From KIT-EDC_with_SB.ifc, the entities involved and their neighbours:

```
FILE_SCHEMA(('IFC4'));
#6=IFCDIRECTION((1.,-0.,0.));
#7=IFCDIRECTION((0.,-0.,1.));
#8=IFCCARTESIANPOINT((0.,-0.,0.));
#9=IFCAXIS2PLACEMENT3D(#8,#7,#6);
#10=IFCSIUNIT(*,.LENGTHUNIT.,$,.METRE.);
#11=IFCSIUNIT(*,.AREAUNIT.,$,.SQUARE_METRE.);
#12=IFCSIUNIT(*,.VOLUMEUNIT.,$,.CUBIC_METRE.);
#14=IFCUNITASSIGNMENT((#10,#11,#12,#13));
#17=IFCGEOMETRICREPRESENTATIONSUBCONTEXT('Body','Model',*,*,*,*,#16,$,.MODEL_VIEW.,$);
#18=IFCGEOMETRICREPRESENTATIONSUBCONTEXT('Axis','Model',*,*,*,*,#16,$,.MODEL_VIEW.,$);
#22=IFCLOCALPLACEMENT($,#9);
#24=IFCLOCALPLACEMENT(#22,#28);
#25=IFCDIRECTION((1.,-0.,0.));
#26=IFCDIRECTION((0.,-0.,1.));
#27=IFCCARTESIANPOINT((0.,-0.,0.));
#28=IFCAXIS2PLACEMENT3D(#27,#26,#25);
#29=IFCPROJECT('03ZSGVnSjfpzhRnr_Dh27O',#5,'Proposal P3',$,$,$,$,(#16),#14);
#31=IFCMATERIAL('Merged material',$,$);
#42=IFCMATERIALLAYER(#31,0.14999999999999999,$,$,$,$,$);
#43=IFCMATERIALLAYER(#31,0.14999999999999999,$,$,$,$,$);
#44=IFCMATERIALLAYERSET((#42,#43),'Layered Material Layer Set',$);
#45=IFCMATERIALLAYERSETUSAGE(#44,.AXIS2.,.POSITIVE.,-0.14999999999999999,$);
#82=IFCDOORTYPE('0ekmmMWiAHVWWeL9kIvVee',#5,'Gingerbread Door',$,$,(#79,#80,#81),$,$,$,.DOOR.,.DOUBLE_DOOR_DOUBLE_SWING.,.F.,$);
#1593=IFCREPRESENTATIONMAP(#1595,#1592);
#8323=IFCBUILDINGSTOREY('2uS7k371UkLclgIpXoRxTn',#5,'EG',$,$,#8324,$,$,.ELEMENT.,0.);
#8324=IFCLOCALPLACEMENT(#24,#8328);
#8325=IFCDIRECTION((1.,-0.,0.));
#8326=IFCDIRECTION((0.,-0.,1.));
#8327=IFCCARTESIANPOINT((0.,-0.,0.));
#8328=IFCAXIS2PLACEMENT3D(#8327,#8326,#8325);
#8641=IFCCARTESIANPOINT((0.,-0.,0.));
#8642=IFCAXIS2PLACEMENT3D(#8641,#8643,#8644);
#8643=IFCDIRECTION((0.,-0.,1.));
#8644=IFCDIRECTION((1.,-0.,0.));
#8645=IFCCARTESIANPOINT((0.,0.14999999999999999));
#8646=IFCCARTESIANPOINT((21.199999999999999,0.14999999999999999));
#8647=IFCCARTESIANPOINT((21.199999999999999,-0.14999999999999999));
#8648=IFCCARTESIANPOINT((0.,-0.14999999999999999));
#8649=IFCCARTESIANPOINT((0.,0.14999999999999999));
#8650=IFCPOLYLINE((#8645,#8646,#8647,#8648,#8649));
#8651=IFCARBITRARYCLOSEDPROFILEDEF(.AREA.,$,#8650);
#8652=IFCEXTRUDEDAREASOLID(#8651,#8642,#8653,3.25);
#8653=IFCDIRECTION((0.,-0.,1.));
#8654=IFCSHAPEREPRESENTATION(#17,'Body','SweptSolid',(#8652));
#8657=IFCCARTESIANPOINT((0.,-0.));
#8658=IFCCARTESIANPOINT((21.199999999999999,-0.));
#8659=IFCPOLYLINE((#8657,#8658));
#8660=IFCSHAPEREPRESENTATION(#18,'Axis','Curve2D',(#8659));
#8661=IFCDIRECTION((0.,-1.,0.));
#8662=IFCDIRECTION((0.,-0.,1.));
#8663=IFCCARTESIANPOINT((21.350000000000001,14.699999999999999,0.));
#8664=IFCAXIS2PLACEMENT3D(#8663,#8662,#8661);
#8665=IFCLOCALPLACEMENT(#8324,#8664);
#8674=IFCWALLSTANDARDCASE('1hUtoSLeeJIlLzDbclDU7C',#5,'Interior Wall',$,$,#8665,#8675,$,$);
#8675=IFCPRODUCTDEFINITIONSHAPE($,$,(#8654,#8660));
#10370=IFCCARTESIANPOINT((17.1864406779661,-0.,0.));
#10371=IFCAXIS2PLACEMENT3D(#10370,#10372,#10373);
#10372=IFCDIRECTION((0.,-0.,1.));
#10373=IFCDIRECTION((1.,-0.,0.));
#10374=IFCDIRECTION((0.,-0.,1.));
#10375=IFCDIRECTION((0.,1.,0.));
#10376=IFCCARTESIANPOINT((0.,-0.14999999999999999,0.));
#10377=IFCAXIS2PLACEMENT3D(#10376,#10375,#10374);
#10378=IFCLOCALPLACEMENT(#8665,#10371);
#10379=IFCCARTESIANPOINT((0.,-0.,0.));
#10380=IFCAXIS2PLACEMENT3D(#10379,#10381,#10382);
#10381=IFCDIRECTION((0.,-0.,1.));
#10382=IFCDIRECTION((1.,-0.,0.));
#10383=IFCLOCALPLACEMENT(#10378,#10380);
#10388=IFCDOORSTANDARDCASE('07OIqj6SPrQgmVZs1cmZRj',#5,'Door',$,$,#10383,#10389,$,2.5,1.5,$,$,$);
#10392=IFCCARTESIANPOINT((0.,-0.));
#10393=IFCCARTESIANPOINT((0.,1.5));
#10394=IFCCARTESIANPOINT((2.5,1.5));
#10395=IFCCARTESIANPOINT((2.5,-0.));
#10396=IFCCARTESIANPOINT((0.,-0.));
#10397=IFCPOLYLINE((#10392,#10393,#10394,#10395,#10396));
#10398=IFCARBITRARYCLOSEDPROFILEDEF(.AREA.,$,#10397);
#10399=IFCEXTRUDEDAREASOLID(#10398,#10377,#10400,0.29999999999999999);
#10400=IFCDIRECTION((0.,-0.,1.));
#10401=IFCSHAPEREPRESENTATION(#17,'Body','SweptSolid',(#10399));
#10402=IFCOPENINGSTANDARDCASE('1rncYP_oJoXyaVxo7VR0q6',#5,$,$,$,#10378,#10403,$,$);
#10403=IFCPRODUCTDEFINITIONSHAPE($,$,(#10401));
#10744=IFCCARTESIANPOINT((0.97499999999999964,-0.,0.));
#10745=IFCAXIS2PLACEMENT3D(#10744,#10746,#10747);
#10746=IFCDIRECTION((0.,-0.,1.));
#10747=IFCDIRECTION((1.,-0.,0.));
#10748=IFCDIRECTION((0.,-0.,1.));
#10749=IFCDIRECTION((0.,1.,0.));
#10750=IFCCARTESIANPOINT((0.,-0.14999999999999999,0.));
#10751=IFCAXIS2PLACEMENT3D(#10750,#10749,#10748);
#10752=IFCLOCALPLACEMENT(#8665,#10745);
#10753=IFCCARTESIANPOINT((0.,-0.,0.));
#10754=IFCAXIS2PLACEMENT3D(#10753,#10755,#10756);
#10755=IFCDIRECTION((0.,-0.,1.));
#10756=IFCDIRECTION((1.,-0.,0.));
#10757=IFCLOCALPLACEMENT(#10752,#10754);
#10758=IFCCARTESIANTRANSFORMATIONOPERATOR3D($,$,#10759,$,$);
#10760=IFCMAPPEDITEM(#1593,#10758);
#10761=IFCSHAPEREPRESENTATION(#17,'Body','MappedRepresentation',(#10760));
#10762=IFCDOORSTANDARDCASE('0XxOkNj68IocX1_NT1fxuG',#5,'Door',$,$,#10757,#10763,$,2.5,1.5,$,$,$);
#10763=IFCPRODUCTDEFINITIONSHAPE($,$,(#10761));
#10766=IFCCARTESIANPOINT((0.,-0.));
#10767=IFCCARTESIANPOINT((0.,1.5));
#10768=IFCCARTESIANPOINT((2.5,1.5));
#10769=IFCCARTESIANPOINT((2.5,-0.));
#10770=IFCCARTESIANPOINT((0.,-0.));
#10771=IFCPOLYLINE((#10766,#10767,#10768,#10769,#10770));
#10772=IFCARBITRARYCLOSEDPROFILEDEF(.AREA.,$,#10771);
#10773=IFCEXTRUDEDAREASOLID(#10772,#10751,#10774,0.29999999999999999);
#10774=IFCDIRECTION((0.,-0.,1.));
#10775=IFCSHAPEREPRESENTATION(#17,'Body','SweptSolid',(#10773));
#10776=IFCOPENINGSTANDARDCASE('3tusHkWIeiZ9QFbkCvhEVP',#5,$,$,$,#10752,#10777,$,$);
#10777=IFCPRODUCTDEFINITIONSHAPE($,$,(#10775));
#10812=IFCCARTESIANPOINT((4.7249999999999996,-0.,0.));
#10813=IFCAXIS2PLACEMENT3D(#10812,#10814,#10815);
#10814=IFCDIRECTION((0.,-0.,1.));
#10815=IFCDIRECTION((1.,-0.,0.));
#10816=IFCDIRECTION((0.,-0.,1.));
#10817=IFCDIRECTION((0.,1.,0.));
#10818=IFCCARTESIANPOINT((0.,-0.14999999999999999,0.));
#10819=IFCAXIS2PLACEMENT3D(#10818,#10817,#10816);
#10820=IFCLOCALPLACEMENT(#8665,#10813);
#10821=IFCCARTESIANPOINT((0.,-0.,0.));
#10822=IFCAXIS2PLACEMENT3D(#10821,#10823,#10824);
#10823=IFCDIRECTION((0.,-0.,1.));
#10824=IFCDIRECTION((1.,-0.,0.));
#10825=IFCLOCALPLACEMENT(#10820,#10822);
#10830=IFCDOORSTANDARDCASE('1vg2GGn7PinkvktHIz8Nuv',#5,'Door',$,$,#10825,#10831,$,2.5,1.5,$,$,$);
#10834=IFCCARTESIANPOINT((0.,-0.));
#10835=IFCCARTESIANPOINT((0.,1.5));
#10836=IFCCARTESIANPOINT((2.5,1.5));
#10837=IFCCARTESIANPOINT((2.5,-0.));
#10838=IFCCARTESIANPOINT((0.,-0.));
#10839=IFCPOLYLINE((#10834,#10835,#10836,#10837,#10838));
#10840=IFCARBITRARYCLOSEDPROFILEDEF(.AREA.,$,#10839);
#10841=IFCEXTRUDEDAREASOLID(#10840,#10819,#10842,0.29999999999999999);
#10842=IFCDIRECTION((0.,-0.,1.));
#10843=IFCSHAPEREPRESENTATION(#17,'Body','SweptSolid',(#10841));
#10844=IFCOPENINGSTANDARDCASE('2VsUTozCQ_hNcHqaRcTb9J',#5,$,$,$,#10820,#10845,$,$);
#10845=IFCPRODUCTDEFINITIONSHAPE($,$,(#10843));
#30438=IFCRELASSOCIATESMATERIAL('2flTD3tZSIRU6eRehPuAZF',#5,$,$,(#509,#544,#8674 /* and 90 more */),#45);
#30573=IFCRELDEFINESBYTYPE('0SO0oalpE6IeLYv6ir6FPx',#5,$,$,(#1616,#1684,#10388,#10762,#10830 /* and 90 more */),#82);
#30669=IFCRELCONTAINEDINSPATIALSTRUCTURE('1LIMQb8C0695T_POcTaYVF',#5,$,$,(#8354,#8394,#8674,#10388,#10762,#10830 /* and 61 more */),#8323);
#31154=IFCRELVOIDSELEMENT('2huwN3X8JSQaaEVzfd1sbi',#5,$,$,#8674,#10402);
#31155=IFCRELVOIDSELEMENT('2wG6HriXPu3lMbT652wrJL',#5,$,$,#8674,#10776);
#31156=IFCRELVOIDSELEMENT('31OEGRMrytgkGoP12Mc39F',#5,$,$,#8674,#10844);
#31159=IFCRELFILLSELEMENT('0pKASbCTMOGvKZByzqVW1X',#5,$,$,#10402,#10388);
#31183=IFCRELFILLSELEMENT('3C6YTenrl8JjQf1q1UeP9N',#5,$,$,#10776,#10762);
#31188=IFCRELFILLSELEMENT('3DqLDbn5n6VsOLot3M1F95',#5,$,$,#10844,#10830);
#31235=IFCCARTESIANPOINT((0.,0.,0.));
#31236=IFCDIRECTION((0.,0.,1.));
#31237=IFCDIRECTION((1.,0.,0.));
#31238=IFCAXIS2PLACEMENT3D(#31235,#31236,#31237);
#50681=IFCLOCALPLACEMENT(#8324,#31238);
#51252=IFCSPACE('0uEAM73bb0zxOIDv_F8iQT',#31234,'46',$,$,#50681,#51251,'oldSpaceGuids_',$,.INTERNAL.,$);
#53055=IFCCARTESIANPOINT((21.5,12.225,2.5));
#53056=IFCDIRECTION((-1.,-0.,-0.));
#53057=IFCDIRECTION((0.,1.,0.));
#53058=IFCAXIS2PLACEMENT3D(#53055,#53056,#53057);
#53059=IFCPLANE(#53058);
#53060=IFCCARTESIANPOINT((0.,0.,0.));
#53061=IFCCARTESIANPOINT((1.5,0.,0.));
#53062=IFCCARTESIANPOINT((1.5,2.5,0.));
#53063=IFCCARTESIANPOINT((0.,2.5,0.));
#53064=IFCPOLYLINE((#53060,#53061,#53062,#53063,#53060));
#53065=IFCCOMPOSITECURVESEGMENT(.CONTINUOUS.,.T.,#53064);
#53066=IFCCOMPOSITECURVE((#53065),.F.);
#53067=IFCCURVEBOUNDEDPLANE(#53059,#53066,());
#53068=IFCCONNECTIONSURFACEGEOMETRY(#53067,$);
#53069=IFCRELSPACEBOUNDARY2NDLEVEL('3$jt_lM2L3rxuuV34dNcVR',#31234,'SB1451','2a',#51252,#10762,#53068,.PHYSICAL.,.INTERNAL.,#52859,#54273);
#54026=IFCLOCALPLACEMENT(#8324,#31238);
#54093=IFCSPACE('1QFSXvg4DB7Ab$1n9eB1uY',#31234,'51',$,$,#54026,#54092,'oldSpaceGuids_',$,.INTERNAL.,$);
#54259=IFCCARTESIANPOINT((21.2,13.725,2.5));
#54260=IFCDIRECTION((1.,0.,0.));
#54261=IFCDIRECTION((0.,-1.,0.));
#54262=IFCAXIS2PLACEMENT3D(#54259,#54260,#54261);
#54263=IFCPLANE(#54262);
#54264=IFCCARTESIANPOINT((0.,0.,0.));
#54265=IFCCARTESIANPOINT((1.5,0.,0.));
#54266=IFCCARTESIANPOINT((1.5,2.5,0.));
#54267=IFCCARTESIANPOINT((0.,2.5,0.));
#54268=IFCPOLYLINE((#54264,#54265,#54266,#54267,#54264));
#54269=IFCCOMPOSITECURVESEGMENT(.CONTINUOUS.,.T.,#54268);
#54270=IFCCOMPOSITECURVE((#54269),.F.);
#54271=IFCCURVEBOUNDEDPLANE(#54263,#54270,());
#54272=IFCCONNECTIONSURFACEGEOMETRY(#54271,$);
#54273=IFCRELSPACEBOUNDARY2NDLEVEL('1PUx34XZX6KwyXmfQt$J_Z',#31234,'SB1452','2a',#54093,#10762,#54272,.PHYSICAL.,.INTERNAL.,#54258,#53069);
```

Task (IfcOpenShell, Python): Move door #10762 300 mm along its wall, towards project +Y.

```python
import numpy as np
import ifcopenshell
import ifcopenshell.api.geometry
import ifcopenshell.util.placement

model = ifcopenshell.open("KIT-EDC_with_SB.ifc")

door = model.by_guid("0XxOkNj68IocX1_NT1fxuG")
opening = door.FillsVoids[0].RelatingOpeningElement
wall = opening.VoidsElements[0].RelatingBuildingElement

wall_matrix = ifcopenshell.util.placement.get_local_placement(wall.ObjectPlacement)
shift = wall_matrix[:3, 0] * -0.3
before = ifcopenshell.util.placement.get_local_placement(door.ObjectPlacement)[:3, 3].copy()

# The door is placed relative to its opening, so it follows when the opening moves.
matrix = ifcopenshell.util.placement.get_local_placement(opening.ObjectPlacement)
matrix[:3, 3] += shift
ifcopenshell.api.geometry.edit_object_placement(
    model, product=opening, matrix=matrix, is_si=False, should_transform_children=True
)

# Space boundary surfaces are stored in each space's coordinates; move them too.
for rel in door.ProvidesBoundaries:
    if not rel.ConnectionGeometry:
        continue
    surface = rel.ConnectionGeometry.SurfaceOnRelatingElement.BasisSurface
    space_matrix = ifcopenshell.util.placement.get_local_placement(rel.RelatingSpace.ObjectPlacement)
    point = np.array(surface.Position.Location.Coordinates) + space_matrix[:3, :3].T @ shift
    surface.Position = model.createIfcAxis2Placement3D(
        model.createIfcCartesianPoint(point.tolist()), surface.Position.Axis, surface.Position.RefDirection
    )

after = ifcopenshell.util.placement.get_local_placement(door.ObjectPlacement)[:3, 3]
print("door moved by", (after - before).round(3) + 0.0)

model.write("KIT-EDC_with_SB_v2.ifc")
```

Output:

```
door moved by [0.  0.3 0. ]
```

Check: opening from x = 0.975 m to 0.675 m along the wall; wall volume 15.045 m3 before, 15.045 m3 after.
